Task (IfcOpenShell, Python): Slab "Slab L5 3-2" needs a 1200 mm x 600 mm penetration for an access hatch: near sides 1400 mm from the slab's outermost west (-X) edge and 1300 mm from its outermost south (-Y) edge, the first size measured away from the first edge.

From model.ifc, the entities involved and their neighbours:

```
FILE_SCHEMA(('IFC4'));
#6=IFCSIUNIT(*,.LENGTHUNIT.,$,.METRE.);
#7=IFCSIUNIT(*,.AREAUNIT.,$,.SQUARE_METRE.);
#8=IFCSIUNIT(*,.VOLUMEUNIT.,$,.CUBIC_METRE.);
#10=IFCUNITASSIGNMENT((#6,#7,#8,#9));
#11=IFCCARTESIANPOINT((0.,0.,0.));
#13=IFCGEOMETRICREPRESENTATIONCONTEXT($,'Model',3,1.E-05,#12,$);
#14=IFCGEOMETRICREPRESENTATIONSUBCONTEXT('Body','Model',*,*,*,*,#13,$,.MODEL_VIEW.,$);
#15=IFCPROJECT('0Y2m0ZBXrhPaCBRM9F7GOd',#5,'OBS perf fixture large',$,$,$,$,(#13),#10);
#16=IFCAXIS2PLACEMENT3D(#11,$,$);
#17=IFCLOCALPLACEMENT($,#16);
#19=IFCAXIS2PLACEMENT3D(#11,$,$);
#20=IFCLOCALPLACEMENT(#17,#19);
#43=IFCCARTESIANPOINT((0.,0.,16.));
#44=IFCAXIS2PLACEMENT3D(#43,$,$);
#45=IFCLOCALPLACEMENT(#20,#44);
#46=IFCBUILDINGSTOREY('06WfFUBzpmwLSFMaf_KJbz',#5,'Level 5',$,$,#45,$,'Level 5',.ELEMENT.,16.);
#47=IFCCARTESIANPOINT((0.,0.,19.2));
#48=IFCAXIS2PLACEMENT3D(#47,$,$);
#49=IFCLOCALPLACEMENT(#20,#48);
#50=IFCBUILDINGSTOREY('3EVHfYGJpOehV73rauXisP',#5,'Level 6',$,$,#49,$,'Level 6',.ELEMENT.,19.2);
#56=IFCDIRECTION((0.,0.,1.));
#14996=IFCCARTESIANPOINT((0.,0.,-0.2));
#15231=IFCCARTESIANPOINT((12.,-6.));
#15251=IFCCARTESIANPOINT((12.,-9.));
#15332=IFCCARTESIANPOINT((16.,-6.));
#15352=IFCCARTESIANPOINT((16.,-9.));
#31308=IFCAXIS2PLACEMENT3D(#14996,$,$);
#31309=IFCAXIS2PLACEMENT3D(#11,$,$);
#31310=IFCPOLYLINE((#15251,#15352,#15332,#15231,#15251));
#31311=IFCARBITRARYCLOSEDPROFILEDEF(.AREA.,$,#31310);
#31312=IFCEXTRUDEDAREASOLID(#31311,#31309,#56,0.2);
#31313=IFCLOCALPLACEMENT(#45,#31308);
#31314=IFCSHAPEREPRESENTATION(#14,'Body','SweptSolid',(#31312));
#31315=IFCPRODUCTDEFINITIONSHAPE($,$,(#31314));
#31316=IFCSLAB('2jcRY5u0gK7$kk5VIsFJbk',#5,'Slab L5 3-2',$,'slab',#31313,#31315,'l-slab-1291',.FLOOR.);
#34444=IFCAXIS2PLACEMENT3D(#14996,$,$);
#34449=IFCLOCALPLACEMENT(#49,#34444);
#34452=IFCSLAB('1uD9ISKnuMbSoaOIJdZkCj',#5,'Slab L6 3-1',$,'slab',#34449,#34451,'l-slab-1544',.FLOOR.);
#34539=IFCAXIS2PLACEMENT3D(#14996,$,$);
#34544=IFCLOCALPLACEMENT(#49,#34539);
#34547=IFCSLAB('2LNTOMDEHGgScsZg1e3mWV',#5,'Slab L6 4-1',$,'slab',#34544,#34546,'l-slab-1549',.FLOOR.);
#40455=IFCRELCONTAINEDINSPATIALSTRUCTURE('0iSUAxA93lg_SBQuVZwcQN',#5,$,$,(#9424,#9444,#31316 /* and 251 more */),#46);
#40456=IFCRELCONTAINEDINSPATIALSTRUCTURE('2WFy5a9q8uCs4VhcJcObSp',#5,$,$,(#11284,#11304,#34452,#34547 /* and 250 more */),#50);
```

```python
import numpy as np
import ifcopenshell
import ifcopenshell.api.feature
import ifcopenshell.api.geometry
import ifcopenshell.api.root
import ifcopenshell.geom
import ifcopenshell.util.placement
import ifcopenshell.util.representation
import ifcopenshell.util.shape
import ifcopenshell.util.unit

model = ifcopenshell.open("model.ifc")
unit_scale = ifcopenshell.util.unit.calculate_unit_scale(model)
settings = ifcopenshell.geom.settings()


def volume(element):
    """Net volume in cubic metres, openings subtracted."""
    shape = ifcopenshell.geom.create_shape(settings, element)
    return ifcopenshell.util.shape.get_volume(shape.geometry)


slab = model.by_guid("2jcRY5u0gK7$kk5VIsFJbk")
before = volume(slab)

# Extent in the slab's own axes, in metres. The edges named are its -X and -Y sides.
slab_shape = ifcopenshell.geom.create_shape(settings, slab)
vertices = ifcopenshell.util.shape.get_vertices(slab_shape.geometry)
x_min, y_min, bottom = vertices.min(axis=0)
top = vertices[:, 2].max()

opening = ifcopenshell.api.root.create_entity(model, ifc_class="IfcOpeningElement", name="Access hatch opening", predefined_type="OPENING")
context = ifcopenshell.util.representation.get_context(model, "Model", "Body", "MODEL_VIEW")
width, depth = 1.2, 0.6
outline = [(0.0, 0.0), (width, 0.0), (width, depth), (0.0, depth), (0.0, 0.0)]
# Overshoot both faces by 50 mm so the cut is clean.
shape = ifcopenshell.api.geometry.add_slab_representation(
    model, context=context, depth=top - bottom + 0.1, polyline=outline
)
ifcopenshell.api.geometry.assign_representation(model, product=opening, representation=shape)

matrix = ifcopenshell.util.placement.get_local_placement(slab.ObjectPlacement)
matrix[:, 3] = matrix @ np.append(np.array([x_min + 1.4, y_min + 1.3, bottom - 0.05]) / unit_scale, 1.0)
ifcopenshell.api.geometry.edit_object_placement(model, product=opening, matrix=matrix, is_si=False)
ifcopenshell.api.feature.add_feature(model, feature=opening, element=slab)

after = volume(slab)

print(f"slab volume {before:.3f} -> {after:.3f} m3")

model.write("model_updated.ifc")
```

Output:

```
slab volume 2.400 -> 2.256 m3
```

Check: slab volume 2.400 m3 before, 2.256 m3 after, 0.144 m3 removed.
